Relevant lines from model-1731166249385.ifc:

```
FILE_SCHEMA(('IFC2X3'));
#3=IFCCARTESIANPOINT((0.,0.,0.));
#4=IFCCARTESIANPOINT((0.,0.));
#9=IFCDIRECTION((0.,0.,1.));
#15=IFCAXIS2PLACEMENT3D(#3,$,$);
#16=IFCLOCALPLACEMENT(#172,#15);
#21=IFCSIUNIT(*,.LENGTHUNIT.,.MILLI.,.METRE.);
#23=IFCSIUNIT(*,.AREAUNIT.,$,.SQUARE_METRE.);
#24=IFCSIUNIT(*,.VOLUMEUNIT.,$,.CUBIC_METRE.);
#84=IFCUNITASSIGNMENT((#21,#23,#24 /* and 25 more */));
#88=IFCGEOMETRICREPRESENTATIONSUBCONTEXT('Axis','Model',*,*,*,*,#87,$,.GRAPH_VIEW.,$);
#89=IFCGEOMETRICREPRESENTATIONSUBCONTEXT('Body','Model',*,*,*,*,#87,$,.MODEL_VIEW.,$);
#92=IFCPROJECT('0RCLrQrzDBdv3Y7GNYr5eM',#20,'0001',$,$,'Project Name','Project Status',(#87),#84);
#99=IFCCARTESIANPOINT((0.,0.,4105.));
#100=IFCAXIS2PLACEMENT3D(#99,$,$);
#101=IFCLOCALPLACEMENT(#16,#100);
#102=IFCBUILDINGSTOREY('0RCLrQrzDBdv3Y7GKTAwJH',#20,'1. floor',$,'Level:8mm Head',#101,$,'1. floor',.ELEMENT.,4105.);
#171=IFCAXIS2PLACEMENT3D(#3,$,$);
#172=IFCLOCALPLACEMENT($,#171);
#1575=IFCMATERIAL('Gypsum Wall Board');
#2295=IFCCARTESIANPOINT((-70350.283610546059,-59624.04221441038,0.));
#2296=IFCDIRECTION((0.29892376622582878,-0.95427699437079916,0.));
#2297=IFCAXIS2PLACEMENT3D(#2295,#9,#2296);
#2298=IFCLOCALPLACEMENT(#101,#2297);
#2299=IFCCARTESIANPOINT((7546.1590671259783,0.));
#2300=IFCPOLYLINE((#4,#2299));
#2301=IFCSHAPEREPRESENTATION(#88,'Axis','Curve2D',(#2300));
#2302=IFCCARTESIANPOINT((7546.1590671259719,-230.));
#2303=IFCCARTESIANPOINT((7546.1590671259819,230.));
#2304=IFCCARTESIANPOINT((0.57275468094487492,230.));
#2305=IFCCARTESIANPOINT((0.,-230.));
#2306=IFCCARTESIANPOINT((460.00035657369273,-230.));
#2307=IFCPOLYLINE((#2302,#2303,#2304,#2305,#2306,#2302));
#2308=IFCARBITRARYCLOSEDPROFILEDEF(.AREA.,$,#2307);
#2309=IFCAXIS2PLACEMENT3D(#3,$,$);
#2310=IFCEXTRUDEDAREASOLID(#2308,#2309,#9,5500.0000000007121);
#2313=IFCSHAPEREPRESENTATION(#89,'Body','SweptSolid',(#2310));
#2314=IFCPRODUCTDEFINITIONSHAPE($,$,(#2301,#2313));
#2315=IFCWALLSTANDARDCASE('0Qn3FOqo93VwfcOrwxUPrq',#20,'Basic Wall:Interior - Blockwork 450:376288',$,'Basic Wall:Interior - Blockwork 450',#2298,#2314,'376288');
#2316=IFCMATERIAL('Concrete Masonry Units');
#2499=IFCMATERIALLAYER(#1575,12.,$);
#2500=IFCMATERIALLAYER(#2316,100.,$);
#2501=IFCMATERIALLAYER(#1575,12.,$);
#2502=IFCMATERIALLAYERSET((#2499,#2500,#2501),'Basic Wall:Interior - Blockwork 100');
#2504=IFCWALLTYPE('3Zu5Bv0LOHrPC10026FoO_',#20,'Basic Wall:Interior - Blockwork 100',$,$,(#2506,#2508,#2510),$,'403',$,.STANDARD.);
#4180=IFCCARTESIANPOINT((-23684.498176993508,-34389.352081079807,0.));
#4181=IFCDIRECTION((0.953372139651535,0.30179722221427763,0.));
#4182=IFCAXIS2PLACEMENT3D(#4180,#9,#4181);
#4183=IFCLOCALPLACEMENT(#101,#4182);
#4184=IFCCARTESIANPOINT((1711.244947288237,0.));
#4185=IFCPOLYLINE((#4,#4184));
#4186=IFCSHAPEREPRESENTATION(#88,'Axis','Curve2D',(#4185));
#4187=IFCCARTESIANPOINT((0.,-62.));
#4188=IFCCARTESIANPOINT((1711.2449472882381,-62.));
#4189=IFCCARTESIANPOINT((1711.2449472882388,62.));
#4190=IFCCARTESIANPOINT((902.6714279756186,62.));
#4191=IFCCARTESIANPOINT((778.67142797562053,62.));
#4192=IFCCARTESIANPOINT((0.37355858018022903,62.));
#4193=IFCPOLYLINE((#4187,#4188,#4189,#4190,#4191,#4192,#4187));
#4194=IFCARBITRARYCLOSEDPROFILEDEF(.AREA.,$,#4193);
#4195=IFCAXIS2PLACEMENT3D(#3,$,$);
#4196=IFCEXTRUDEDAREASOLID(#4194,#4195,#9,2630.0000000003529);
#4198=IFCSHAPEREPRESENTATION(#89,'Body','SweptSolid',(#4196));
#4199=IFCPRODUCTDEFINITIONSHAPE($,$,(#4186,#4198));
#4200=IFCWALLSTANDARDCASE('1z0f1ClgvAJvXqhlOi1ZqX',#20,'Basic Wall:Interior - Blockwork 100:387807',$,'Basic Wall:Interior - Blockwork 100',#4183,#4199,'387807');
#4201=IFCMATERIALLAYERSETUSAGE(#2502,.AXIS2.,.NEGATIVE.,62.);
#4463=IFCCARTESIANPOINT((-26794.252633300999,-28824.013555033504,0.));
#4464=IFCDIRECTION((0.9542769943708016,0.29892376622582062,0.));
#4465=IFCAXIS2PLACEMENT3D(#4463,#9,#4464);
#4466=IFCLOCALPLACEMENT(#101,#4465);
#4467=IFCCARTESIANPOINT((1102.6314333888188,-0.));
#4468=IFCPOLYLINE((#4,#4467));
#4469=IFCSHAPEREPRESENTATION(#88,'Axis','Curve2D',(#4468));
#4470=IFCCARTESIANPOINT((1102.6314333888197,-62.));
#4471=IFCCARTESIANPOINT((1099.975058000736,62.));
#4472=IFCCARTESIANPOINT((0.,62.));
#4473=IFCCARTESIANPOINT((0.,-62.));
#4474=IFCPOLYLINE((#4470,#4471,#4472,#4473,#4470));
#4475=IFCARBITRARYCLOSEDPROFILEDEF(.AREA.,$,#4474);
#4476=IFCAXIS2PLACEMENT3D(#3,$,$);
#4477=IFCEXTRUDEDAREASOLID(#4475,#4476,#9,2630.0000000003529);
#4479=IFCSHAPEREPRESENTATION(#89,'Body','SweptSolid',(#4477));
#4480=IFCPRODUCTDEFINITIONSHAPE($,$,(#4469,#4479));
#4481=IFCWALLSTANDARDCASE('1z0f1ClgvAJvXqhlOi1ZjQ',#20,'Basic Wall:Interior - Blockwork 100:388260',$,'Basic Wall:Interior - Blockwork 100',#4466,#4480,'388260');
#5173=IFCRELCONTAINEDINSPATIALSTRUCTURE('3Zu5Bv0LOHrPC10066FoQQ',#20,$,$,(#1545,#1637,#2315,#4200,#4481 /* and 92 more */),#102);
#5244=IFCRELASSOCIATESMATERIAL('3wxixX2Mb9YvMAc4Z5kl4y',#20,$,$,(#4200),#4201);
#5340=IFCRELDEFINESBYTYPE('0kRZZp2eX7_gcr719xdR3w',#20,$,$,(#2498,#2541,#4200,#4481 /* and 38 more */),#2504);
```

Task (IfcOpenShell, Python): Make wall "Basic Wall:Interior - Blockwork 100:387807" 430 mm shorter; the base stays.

```python
import ifcopenshell
import ifcopenshell.geom
import ifcopenshell.util.representation
import ifcopenshell.util.shape
import ifcopenshell.util.unit

model = ifcopenshell.open("model-1731166249385.ifc")
unit_scale = ifcopenshell.util.unit.calculate_unit_scale(model)
settings = ifcopenshell.geom.settings()


def volume(element):
    """Net volume in cubic metres, openings subtracted."""
    shape = ifcopenshell.geom.create_shape(settings, element)
    return ifcopenshell.util.shape.get_volume(shape.geometry)


wall = model.by_guid("1z0f1ClgvAJvXqhlOi1ZqX")
before = volume(wall)

body = ifcopenshell.util.representation.get_representation(wall, "Model", "Body")
solid = body.Items[0]
old_height = solid.Depth
solid.Depth -= 0.43 / unit_scale
after = volume(wall)

print(f"height {old_height:g} -> {solid.Depth:g}, volume {before:.3f} -> {after:.3f} m3")

model.write("model-1731166249385-out.ifc")
```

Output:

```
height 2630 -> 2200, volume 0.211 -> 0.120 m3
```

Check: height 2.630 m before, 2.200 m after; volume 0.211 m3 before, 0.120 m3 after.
